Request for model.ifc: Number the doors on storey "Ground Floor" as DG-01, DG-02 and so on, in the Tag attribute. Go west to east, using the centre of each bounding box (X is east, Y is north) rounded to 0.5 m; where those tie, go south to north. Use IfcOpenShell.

First a look at what the model holds.

```python
import ifcopenshell
import ifcopenshell.util.element
import ifcopenshell.util.placement

model = ifcopenshell.open("model.ifc")
print(model.schema)
storey = next(s for s in model.by_type("IfcBuildingStorey") if s.Name == "Ground Floor")
doors = [e for e in ifcopenshell.util.element.get_decomposition(storey) if e.is_a("IfcDoor")]
for e in sorted(doors, key=lambda e: e.id()):
    origin = ifcopenshell.util.placement.get_local_placement(e.ObjectPlacement)[:3, 3]
    print(e.id(), e.Tag, e.Name, origin.round(2) + 0.0, sep=" | ")
```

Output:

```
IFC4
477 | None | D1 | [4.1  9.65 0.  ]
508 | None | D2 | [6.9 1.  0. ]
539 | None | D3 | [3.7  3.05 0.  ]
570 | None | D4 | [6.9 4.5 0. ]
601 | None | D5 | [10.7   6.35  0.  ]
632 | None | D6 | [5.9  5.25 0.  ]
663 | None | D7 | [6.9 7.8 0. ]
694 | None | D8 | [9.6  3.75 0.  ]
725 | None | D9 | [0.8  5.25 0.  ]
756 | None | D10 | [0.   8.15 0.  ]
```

```python
import ifcopenshell
import ifcopenshell.geom
import ifcopenshell.util.element
import ifcopenshell.util.shape

model = ifcopenshell.open("model.ifc")
settings = ifcopenshell.geom.settings()
settings.set("use-world-coords", True)


def centre(element):
    shape = ifcopenshell.geom.create_shape(settings, element)
    return ifcopenshell.util.shape.get_bbox_centroid(shape.geometry)


storey = next(s for s in model.by_type("IfcBuildingStorey") if s.Name == "Ground Floor")
doors = [e for e in ifcopenshell.util.element.get_decomposition(storey) if e.is_a("IfcDoor")]

# Insertion points can sit at a corner or the storey origin, so sort by the geometry (in metres).
centres = {e: centre(e) for e in doors}
doors.sort(key=lambda e: (round(centres[e][0] / 0.5), centres[e][1]))

for i, e in enumerate(doors, start=1):
    number = f"DG-{i:02d}"
    e.Tag = number
    print(e.id(), number)

model.write("model_edited.ifc")
```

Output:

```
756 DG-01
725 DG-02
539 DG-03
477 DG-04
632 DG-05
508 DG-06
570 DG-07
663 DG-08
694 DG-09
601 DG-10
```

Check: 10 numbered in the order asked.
